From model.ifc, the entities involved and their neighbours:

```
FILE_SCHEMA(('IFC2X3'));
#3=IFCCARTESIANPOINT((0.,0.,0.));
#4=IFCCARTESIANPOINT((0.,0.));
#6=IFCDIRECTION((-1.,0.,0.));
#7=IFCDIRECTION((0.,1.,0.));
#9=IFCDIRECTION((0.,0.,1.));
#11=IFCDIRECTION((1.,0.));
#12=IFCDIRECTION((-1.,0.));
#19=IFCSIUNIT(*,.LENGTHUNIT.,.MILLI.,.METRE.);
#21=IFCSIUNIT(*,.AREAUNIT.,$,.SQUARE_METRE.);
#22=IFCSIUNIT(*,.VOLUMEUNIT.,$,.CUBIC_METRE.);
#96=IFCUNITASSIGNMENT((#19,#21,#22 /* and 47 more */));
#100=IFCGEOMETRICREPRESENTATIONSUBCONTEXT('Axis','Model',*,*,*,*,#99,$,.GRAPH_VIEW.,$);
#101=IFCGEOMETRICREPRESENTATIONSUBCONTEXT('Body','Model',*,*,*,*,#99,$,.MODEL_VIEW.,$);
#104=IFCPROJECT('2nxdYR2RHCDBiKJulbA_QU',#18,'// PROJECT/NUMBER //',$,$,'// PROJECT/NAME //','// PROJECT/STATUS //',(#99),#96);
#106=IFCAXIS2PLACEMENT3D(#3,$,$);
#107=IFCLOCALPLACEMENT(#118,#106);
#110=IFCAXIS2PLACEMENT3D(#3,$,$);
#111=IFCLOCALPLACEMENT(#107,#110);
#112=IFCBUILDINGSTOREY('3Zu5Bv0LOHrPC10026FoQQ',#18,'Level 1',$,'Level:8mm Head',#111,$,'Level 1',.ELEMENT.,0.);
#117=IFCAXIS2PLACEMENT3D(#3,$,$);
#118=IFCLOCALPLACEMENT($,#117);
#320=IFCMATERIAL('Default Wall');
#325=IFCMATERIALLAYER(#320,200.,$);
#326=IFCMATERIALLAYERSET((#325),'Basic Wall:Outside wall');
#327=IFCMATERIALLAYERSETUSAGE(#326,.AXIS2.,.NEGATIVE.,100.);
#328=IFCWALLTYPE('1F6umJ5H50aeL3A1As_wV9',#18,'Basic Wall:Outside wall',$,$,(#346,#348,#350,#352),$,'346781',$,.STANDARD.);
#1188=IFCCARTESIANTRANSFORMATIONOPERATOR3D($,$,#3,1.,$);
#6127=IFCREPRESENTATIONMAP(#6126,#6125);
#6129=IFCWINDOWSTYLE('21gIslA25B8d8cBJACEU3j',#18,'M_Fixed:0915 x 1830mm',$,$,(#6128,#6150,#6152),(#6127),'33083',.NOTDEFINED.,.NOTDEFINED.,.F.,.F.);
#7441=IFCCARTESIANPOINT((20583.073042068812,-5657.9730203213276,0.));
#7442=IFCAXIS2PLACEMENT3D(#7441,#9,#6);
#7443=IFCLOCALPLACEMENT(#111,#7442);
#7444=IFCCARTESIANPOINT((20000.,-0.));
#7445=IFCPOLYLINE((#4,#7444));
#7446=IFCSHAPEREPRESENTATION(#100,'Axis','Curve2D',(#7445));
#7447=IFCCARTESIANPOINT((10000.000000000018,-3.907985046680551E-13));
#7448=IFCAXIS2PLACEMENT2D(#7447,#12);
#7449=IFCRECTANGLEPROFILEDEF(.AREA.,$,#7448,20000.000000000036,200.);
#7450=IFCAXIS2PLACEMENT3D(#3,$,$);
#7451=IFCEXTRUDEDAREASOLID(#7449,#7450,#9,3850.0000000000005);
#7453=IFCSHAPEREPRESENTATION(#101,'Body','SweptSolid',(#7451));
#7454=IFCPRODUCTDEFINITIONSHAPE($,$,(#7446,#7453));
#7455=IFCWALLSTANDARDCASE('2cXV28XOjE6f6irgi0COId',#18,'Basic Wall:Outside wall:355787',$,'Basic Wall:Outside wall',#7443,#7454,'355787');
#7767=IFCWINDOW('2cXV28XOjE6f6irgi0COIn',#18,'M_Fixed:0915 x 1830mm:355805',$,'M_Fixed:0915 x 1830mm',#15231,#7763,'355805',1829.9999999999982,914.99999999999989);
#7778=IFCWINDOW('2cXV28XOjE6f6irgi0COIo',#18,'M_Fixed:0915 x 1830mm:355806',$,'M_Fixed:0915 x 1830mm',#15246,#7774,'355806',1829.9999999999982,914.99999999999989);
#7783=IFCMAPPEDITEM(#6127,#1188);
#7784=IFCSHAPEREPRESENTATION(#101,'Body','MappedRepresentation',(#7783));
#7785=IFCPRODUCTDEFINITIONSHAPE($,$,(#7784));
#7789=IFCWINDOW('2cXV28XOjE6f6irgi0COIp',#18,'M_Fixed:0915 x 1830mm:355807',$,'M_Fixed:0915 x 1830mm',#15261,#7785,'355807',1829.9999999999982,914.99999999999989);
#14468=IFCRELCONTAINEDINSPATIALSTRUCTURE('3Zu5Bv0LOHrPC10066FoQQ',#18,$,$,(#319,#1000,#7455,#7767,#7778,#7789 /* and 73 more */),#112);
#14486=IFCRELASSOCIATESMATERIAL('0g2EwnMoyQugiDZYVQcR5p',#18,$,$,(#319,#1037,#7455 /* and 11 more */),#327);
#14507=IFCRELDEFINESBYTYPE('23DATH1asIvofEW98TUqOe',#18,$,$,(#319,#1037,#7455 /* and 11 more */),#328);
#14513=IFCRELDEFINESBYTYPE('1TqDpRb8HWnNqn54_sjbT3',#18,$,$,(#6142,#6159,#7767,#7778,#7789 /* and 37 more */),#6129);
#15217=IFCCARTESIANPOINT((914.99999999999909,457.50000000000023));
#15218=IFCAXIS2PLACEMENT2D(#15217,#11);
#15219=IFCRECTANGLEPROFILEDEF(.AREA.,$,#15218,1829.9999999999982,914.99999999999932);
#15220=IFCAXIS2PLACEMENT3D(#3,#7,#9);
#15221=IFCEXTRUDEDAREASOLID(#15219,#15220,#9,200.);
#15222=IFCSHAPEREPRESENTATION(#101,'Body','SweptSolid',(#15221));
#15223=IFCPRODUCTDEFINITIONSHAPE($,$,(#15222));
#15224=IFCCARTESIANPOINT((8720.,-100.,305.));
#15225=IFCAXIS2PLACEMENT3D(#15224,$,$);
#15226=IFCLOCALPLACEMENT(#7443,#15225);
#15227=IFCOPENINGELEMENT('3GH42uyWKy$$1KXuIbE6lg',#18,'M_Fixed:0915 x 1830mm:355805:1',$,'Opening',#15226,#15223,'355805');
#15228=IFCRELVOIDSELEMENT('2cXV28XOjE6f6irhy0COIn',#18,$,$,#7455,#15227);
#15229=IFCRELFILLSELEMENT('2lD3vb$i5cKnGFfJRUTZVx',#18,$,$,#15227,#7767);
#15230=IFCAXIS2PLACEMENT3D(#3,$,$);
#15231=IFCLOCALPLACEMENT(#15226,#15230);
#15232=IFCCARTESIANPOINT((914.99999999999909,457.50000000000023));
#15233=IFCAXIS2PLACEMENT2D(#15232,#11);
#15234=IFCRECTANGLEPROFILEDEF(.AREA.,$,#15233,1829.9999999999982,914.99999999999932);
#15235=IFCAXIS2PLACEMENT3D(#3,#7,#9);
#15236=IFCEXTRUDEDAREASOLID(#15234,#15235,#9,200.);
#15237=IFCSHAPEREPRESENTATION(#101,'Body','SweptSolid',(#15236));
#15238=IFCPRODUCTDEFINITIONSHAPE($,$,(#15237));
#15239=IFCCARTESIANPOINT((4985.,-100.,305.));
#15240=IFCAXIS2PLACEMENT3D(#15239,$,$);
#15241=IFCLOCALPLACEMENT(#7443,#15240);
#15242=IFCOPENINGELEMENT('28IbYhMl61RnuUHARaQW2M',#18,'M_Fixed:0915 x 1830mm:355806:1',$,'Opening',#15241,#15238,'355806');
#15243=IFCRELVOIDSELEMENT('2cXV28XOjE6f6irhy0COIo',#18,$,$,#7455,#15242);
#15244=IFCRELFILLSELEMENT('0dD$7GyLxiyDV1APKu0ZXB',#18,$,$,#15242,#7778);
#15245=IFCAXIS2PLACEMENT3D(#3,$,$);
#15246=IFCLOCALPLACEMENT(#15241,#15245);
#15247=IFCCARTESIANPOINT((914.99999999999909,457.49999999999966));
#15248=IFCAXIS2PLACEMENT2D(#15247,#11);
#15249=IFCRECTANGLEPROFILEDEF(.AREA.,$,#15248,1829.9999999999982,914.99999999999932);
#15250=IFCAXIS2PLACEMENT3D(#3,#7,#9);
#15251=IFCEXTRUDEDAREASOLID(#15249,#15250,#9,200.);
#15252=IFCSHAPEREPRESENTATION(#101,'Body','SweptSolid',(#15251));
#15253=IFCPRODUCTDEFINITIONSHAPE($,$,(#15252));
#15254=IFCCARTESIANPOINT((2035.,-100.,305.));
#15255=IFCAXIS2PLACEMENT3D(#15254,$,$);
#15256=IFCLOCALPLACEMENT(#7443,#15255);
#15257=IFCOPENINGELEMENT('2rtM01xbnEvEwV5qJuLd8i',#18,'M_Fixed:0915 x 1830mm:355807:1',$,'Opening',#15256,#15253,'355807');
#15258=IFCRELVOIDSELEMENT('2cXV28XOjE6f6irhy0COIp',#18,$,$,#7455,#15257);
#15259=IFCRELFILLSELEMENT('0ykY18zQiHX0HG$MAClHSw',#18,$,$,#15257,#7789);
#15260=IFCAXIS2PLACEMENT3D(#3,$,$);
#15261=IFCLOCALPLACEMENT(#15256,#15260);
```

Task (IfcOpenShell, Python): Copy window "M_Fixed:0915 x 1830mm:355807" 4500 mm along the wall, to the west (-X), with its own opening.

```python
import ifcopenshell
import ifcopenshell.api.feature
import ifcopenshell.api.geometry
import ifcopenshell.api.root
import ifcopenshell.geom
import ifcopenshell.util.element
import ifcopenshell.util.placement
import ifcopenshell.util.shape
import ifcopenshell.util.unit

model = ifcopenshell.open("model.ifc")
unit_scale = ifcopenshell.util.unit.calculate_unit_scale(model)
settings = ifcopenshell.geom.settings()


def volume(element):
    """Net volume in cubic metres, openings subtracted."""
    shape = ifcopenshell.geom.create_shape(settings, element)
    return ifcopenshell.util.shape.get_volume(shape.geometry)


def reuse_history(source, copy):
    """copy_class also copies each property set's owner history, people and application; keep the originals."""
    for rel in copy.IsDefinedBy:
        if rel.is_a("IfcRelDefinesByProperties") and (history := rel.RelatingPropertyDefinition.OwnerHistory):
            rel.RelatingPropertyDefinition.OwnerHistory = source.OwnerHistory
            ifcopenshell.util.element.remove_deep2(model, history)


window = model.by_guid("2cXV28XOjE6f6irgi0COIp")
opening = window.FillsVoids[0].RelatingOpeningElement
wall = opening.VoidsElements[0].RelatingBuildingElement
before = volume(wall)
shift = ifcopenshell.util.placement.get_local_placement(wall.ObjectPlacement)[:3, 0] * 4.5 / unit_scale

# copy_class copies the void relationship, type, container and properties, but no geometry.
new_opening = ifcopenshell.api.root.copy_class(model, product=opening)
new_opening.Representation = ifcopenshell.util.element.copy_deep(
    model, opening.Representation, exclude=["IfcGeometricRepresentationContext", "IfcRepresentationMap"]
)
new_opening.Name = "M_Fixed:0915 x 1830mm"
new_opening.Tag = None
new_window = ifcopenshell.api.root.copy_class(model, product=window)
new_window.Representation = ifcopenshell.util.element.copy_deep(
    model, window.Representation, exclude=["IfcGeometricRepresentationContext", "IfcRepresentationMap"]
)
new_window.Name = "M_Fixed:0915 x 1830mm"
new_window.Tag = None
reuse_history(window, new_window)
fills = ifcopenshell.api.feature.add_filling(model, opening=new_opening, element=new_window)
fills.OwnerHistory = new_window.OwnerHistory  # required in IFC2X3

for old, new in ((opening, new_opening), (window, new_window)):
    matrix = ifcopenshell.util.placement.get_local_placement(old.ObjectPlacement)
    matrix[:3, 3] += shift
    ifcopenshell.api.geometry.edit_object_placement(model, product=new, matrix=matrix, is_si=False)

after = volume(wall)

print(f"wall volume {before:.3f} -> {after:.3f} m3")

model.write("model-out.ifc")
```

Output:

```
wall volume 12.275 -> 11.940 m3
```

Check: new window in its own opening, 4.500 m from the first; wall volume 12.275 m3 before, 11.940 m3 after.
